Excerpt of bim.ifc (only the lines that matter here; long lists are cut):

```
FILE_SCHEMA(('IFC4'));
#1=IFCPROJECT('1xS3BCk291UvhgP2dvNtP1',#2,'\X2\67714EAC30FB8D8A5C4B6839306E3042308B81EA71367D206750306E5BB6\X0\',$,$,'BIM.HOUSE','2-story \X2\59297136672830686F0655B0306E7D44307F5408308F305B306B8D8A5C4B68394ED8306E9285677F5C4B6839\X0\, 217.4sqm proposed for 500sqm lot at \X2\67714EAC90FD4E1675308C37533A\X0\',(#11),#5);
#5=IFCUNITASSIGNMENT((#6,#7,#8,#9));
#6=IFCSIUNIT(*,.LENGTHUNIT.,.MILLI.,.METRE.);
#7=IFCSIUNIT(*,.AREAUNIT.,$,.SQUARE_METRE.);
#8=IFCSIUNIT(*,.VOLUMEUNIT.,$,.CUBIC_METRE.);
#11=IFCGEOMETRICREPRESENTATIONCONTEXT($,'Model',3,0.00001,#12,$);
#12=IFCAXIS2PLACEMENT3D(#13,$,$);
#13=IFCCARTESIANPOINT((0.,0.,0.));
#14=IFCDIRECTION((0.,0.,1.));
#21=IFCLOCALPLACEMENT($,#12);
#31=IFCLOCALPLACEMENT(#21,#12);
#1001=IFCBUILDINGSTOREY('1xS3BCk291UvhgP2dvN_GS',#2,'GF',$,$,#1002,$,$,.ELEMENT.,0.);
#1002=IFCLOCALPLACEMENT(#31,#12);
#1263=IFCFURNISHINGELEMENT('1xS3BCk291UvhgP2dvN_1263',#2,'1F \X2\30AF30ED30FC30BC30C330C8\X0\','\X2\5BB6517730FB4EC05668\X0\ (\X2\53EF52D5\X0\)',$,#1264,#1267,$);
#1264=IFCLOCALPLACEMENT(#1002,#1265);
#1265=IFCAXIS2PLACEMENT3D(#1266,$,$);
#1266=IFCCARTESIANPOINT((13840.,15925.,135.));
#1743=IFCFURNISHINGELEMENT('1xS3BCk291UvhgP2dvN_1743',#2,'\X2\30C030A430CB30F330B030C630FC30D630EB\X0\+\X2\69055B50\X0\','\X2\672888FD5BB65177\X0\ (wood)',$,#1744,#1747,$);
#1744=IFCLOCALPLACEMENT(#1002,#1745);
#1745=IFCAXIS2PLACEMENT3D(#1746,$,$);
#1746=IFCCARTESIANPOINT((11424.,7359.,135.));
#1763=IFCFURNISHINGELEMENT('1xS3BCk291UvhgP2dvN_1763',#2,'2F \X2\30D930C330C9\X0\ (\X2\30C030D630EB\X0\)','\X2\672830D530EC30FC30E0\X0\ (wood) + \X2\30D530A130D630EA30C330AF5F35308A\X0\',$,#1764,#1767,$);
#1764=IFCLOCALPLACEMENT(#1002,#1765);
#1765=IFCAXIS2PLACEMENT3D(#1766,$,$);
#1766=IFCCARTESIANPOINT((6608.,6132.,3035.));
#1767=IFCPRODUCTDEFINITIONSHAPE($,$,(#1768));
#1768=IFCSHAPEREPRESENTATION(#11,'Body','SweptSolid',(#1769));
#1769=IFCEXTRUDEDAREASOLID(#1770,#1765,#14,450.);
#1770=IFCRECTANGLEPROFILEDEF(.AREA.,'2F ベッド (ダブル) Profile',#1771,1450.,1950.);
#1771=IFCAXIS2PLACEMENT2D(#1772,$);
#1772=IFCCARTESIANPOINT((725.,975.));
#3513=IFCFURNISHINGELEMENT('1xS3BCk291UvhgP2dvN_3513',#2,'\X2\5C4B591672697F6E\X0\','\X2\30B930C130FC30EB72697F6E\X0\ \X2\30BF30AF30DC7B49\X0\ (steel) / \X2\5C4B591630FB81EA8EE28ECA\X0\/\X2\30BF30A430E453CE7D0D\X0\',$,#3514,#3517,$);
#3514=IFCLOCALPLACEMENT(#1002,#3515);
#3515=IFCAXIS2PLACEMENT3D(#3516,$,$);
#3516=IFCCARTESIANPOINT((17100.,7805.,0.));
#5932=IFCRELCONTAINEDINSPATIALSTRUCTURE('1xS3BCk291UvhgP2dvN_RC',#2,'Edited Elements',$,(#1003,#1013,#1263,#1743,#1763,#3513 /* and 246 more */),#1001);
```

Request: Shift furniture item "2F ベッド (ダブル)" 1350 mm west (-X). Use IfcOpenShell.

```python
import ifcopenshell
import ifcopenshell.api.geometry
import ifcopenshell.util.placement

model = ifcopenshell.open("bim.ifc")

item = model.by_guid("1xS3BCk291UvhgP2dvN_1763")
matrix = ifcopenshell.util.placement.get_local_placement(item.ObjectPlacement)
matrix[0, 3] -= 1350.0
ifcopenshell.api.geometry.edit_object_placement(model, product=item, matrix=matrix, is_si=False)

print(ifcopenshell.util.placement.get_local_placement(item.ObjectPlacement).round(3) + 0.0)

model.write("bim-out.ifc")
```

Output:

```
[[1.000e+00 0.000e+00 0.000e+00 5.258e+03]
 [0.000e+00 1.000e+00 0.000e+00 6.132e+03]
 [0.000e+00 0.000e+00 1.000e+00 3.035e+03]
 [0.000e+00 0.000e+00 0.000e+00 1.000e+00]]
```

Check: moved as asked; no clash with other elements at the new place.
